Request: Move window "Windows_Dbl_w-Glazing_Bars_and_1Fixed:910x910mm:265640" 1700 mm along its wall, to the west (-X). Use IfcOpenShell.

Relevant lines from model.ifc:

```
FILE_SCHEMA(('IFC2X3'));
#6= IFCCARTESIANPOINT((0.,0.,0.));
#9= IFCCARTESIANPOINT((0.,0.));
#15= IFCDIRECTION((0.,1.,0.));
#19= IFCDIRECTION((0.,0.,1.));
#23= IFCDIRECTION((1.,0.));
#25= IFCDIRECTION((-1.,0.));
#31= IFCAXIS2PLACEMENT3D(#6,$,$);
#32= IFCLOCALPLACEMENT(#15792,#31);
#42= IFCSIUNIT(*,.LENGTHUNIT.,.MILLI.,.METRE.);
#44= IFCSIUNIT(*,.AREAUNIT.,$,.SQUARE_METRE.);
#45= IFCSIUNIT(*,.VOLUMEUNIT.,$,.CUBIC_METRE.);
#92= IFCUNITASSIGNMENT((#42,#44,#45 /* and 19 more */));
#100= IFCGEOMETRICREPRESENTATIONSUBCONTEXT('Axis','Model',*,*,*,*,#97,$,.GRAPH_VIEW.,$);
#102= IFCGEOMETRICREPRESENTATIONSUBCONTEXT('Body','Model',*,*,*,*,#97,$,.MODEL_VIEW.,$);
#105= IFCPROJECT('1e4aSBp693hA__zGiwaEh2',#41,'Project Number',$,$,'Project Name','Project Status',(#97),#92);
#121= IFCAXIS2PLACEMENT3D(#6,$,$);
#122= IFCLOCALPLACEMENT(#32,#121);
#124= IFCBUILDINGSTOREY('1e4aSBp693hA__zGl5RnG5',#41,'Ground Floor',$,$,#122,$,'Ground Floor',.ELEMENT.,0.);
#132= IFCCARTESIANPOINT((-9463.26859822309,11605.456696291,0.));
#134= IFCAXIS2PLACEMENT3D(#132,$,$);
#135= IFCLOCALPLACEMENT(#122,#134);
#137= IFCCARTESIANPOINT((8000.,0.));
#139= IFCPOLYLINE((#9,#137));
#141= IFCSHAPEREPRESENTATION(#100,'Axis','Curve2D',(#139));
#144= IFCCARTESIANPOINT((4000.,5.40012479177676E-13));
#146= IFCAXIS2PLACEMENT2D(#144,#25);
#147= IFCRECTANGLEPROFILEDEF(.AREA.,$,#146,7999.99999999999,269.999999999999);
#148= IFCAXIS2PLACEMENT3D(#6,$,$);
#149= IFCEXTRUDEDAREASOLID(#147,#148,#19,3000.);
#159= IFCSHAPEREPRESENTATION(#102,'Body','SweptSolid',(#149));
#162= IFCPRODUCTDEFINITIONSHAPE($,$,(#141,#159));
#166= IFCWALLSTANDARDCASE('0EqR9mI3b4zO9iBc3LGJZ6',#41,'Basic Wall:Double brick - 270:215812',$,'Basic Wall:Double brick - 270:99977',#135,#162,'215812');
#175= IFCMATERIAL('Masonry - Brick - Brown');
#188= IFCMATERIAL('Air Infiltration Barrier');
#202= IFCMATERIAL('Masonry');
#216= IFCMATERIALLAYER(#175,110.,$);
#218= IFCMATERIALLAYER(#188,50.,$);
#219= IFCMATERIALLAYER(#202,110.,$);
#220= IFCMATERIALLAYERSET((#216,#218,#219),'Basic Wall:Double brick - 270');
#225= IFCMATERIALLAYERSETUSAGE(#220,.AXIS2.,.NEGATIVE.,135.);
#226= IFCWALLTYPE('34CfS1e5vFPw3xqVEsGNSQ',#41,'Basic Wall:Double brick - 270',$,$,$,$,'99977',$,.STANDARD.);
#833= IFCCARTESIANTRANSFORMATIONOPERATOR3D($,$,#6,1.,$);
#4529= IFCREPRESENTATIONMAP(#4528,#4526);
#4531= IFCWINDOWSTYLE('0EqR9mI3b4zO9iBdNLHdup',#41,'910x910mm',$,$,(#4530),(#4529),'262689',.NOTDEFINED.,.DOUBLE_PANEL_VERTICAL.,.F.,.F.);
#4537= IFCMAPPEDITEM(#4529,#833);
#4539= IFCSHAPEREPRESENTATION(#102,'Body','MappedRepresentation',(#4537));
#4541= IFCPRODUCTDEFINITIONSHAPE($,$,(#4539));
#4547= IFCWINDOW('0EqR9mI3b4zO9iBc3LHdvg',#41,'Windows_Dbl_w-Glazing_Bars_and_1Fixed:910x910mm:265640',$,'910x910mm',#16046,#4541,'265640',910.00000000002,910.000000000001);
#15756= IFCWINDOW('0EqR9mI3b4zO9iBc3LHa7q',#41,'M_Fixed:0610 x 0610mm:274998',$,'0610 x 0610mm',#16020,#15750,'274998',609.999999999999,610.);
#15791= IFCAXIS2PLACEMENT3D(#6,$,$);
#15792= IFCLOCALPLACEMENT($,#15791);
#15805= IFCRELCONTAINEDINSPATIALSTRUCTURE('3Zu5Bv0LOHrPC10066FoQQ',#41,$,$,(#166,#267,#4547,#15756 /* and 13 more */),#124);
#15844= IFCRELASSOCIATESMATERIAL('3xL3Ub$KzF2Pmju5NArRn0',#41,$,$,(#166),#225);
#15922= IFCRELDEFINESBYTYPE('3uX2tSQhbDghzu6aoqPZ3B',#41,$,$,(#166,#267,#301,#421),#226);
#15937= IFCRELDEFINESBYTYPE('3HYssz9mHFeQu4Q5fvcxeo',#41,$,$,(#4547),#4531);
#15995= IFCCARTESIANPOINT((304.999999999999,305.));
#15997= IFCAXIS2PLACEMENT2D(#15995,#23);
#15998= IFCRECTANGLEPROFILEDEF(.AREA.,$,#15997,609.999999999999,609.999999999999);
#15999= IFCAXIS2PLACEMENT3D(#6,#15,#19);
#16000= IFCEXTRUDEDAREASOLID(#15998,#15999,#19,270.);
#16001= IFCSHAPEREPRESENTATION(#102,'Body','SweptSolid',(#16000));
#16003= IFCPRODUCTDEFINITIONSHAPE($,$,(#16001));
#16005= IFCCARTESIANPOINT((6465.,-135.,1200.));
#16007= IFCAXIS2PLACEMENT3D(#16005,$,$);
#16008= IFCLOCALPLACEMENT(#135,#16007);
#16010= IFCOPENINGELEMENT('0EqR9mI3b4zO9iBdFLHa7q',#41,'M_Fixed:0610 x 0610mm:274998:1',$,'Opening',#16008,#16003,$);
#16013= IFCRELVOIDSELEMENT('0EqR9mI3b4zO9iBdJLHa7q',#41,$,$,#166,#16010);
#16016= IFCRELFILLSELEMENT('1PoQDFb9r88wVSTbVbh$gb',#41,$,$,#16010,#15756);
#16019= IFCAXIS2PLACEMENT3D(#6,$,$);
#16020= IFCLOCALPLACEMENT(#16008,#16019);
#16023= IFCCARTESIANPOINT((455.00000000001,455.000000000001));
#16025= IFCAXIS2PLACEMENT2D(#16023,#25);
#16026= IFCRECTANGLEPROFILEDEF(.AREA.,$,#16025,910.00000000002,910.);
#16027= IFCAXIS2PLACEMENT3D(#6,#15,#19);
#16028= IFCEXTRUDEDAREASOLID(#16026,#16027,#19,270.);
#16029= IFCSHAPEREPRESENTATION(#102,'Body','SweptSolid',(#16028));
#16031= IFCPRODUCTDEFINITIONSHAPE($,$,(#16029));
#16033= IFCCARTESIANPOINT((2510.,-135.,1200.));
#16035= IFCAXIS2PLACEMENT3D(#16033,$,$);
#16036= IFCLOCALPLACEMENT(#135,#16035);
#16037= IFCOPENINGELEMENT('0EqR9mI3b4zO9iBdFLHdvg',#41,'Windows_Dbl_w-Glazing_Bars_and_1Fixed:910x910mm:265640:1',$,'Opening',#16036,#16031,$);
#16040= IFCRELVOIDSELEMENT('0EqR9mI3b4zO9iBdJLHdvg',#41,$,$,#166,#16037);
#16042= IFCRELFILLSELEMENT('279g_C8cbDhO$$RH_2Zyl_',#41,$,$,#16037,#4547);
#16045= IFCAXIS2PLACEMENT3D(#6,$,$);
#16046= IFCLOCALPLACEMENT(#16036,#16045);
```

```python
import ifcopenshell
import ifcopenshell.api.geometry
import ifcopenshell.util.placement

model = ifcopenshell.open("model.ifc")

window = model.by_guid("0EqR9mI3b4zO9iBc3LHdvg")
opening = window.FillsVoids[0].RelatingOpeningElement
wall = opening.VoidsElements[0].RelatingBuildingElement

wall_matrix = ifcopenshell.util.placement.get_local_placement(wall.ObjectPlacement)
shift = wall_matrix[:3, 0] * -1700.0
before = ifcopenshell.util.placement.get_local_placement(window.ObjectPlacement)[:3, 3].copy()

# The window is placed relative to its opening, so it follows when the opening moves.
matrix = ifcopenshell.util.placement.get_local_placement(opening.ObjectPlacement)
matrix[:3, 3] += shift
ifcopenshell.api.geometry.edit_object_placement(
    model, product=opening, matrix=matrix, is_si=False, should_transform_children=True
)

after = ifcopenshell.util.placement.get_local_placement(window.ObjectPlacement)[:3, 3]
print("window moved by", (after - before).round(3) + 0.0)

model.write("model_rev.ifc")
```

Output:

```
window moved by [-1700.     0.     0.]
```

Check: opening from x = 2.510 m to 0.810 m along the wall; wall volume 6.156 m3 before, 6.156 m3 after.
